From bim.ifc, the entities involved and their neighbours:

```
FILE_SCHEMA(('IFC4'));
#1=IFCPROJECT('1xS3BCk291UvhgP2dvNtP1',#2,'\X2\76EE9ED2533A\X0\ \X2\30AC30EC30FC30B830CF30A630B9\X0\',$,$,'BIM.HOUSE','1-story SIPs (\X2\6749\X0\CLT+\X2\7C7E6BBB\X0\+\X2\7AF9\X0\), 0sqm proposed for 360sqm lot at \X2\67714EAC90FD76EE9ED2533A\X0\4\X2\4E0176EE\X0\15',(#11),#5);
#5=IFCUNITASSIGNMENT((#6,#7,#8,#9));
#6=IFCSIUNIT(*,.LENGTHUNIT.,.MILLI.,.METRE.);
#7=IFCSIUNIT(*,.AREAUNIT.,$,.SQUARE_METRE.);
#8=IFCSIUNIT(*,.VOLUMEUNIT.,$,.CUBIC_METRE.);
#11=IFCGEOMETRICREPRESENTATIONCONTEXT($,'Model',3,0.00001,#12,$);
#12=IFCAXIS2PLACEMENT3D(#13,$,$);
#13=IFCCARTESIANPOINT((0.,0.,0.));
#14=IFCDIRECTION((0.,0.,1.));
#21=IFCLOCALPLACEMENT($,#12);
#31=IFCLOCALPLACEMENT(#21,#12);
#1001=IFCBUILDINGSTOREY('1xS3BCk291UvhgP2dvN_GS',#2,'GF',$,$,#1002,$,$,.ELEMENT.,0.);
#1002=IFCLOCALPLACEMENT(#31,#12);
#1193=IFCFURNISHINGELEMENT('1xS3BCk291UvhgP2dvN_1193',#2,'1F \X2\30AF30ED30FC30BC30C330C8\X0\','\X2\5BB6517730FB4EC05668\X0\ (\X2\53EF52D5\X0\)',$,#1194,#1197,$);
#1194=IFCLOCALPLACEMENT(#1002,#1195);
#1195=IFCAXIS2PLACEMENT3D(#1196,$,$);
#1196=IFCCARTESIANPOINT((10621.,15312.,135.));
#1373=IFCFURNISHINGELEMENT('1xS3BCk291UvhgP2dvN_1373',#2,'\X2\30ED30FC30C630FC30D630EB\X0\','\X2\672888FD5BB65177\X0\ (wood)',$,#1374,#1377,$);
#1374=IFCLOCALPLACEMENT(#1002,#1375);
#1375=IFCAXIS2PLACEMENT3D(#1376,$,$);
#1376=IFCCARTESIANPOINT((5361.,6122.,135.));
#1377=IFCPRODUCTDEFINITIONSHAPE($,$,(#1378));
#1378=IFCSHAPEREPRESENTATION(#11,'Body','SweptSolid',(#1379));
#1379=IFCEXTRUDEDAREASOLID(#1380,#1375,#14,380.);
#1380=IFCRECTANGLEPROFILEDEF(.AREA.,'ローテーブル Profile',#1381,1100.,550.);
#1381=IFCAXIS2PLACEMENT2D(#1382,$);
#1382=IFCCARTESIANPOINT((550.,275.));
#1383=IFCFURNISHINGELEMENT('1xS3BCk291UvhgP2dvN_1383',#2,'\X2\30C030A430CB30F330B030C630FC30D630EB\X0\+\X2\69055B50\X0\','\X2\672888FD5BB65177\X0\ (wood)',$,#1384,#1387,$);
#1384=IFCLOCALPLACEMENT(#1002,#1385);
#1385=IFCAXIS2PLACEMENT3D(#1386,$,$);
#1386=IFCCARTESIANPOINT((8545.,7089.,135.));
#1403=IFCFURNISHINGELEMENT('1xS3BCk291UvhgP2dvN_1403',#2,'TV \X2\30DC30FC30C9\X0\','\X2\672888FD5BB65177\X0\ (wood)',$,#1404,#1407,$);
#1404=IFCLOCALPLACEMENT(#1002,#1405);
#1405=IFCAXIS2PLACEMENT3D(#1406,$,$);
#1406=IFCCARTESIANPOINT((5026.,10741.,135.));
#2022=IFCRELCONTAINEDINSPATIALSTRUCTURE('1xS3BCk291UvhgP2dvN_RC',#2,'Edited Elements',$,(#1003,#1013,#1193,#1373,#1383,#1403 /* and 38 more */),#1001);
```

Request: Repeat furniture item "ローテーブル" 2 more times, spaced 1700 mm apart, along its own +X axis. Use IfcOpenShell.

```python
import ifcopenshell
import ifcopenshell.api.geometry
import ifcopenshell.api.root
import ifcopenshell.util.element
import ifcopenshell.util.placement

model = ifcopenshell.open("bim.ifc")


def reuse_history(source, copy):
    """copy_class also copies each property set's owner history, people and application; keep the originals."""
    for rel in copy.IsDefinedBy:
        if rel.is_a("IfcRelDefinesByProperties") and (history := rel.RelatingPropertyDefinition.OwnerHistory):
            rel.RelatingPropertyDefinition.OwnerHistory = source.OwnerHistory
            ifcopenshell.util.element.remove_deep2(model, history)


source = model.by_guid("1xS3BCk291UvhgP2dvN_1373")
base = ifcopenshell.util.placement.get_local_placement(source.ObjectPlacement)
step = base[:3, 0] * 1700.0

for i in range(1, 3):
    copy = ifcopenshell.api.root.copy_class(model, product=source)
    copy.Representation = ifcopenshell.util.element.copy_deep(
        model, source.Representation, exclude=["IfcGeometricRepresentationContext", "IfcRepresentationMap"]
    )
    reuse_history(source, copy)
    matrix = base.copy()
    matrix[:3, 3] += i * step
    print("added at", matrix[:3, 3].round(3) + 0.0)
    ifcopenshell.api.geometry.edit_object_placement(model, product=copy, matrix=matrix, is_si=False)

model.write("bim-out.ifc")
```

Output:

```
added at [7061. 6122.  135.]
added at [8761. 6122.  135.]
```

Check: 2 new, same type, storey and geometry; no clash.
